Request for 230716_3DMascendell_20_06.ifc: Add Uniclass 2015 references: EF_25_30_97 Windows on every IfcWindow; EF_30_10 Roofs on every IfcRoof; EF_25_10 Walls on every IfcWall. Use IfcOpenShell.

First a look at what the model holds.

```python
import ifcopenshell

model = ifcopenshell.open("230716_3DMascendell_20_06.ifc")
print(model.schema)
print("classifications:", [c.Name for c in model.by_type("IfcClassification")])
for ifc_class in ("IfcDoor", "IfcRoof", "IfcStair", "IfcWall", "IfcWindow"):
    print(ifc_class, len(model.by_type(ifc_class)))
```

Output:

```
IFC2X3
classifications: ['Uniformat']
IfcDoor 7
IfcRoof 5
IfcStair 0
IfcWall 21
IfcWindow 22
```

```python
import ifcopenshell
import ifcopenshell.api.classification

model = ifcopenshell.open("230716_3DMascendell_20_06.ifc")

# IFC2X3 requires Source and Edition and has no link from the project to the system.
system = model.create_entity("IfcClassification", Source="NBS", Edition="2015", Name="Uniclass 2015")

codes = {
    "IfcWindow": ("EF_25_30_97", "Windows"),
    "IfcRoof": ("EF_30_10", "Roofs"),
    "IfcWall": ("EF_25_10", "Walls"),
}
for ifc_class, (code, name) in codes.items():
    products = model.by_type(ifc_class)
    ifcopenshell.api.classification.add_reference(
        model, products=products, classification=system, identification=code, name=name
    )
    print(code, len(products))

model.write("230716_3DMascendell_20_06_updated.ifc")
```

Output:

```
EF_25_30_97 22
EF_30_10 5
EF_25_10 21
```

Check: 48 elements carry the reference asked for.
